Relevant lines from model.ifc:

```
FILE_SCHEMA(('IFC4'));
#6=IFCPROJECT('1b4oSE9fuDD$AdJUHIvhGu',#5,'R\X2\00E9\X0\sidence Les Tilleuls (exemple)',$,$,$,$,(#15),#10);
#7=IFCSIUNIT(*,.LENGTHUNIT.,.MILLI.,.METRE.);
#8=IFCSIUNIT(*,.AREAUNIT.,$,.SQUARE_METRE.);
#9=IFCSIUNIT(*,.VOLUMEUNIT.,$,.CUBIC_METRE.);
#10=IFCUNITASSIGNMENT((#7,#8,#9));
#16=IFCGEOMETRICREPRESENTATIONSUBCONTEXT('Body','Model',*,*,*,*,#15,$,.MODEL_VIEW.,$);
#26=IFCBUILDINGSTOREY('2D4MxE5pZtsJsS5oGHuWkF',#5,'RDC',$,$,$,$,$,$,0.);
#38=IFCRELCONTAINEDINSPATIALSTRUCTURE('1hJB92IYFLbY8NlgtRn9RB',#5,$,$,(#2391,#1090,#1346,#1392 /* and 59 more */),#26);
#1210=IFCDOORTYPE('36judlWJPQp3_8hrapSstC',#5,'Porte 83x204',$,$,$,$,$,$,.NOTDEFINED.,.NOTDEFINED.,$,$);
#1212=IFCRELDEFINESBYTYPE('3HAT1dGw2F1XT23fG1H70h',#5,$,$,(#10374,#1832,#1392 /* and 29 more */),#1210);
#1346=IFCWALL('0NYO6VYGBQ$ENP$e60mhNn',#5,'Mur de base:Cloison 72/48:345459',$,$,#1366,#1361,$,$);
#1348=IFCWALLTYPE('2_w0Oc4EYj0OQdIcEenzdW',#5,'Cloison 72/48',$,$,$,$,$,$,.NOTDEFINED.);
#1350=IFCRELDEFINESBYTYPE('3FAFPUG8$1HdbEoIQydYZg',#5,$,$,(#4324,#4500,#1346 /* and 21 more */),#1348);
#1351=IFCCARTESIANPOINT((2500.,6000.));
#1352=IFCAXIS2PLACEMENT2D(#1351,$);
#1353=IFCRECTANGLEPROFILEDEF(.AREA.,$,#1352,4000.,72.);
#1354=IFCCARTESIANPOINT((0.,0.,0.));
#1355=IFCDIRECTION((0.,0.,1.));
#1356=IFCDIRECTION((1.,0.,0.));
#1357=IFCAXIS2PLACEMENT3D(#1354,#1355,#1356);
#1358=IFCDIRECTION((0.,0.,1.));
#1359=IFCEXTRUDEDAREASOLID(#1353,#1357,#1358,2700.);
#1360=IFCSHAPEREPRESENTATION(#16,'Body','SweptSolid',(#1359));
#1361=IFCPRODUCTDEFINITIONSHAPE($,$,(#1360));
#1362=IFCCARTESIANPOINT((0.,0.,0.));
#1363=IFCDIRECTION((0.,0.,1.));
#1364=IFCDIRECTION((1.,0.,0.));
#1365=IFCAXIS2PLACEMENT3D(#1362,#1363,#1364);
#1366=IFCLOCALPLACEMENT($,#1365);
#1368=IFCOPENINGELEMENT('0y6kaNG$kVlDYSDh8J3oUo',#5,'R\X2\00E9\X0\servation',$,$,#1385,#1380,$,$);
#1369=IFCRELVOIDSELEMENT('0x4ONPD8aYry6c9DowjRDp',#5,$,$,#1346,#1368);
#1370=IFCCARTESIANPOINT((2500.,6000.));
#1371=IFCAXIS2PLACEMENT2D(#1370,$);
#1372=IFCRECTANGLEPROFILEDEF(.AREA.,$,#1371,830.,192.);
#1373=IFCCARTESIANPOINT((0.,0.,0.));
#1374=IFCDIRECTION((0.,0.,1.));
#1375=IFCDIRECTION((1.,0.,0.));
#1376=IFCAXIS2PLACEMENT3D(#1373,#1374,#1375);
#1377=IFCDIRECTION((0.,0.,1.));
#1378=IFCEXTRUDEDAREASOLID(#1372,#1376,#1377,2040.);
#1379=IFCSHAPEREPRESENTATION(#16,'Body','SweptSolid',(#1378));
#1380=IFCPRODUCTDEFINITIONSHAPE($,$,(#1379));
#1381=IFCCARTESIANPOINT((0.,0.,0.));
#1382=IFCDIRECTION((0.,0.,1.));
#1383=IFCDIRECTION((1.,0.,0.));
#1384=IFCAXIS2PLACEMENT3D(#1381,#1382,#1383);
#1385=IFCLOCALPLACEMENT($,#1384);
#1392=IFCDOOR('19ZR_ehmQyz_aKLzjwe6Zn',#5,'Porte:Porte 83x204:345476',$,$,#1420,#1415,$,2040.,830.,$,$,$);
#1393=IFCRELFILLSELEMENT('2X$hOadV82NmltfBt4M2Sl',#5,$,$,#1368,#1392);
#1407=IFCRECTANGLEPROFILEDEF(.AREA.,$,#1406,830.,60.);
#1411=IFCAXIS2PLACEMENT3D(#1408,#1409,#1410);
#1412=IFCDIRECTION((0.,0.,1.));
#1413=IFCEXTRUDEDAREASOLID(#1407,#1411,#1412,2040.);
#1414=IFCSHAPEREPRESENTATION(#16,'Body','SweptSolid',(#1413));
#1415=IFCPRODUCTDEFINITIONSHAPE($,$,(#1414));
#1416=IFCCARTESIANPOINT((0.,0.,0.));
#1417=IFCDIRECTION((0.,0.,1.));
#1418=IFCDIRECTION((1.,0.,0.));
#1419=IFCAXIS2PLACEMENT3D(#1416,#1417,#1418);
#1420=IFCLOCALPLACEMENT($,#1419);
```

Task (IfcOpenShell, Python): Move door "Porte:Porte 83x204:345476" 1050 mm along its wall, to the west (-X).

```python
import ifcopenshell
import ifcopenshell.api.geometry
import ifcopenshell.util.placement
import ifcopenshell.util.unit

model = ifcopenshell.open("model.ifc")
unit_scale = ifcopenshell.util.unit.calculate_unit_scale(model)

door = model.by_guid("19ZR_ehmQyz_aKLzjwe6Zn")
opening = door.FillsVoids[0].RelatingOpeningElement
wall = opening.VoidsElements[0].RelatingBuildingElement

wall_matrix = ifcopenshell.util.placement.get_local_placement(wall.ObjectPlacement)
shift = wall_matrix[:3, 0] * -1.05 / unit_scale
before = ifcopenshell.util.placement.get_local_placement(door.ObjectPlacement)[:3, 3].copy()

# The door is not placed relative to its opening, so move both.
for product in (opening, door):
    matrix = ifcopenshell.util.placement.get_local_placement(product.ObjectPlacement)
    matrix[:3, 3] += shift
    ifcopenshell.api.geometry.edit_object_placement(model, product=product, matrix=matrix, is_si=False)

after = ifcopenshell.util.placement.get_local_placement(door.ObjectPlacement)[:3, 3]
print("door moved by", (after - before).round(3) + 0.0)

model.write("model_edited.ifc")
```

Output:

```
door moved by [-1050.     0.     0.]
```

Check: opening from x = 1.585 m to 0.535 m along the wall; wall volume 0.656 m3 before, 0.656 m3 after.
